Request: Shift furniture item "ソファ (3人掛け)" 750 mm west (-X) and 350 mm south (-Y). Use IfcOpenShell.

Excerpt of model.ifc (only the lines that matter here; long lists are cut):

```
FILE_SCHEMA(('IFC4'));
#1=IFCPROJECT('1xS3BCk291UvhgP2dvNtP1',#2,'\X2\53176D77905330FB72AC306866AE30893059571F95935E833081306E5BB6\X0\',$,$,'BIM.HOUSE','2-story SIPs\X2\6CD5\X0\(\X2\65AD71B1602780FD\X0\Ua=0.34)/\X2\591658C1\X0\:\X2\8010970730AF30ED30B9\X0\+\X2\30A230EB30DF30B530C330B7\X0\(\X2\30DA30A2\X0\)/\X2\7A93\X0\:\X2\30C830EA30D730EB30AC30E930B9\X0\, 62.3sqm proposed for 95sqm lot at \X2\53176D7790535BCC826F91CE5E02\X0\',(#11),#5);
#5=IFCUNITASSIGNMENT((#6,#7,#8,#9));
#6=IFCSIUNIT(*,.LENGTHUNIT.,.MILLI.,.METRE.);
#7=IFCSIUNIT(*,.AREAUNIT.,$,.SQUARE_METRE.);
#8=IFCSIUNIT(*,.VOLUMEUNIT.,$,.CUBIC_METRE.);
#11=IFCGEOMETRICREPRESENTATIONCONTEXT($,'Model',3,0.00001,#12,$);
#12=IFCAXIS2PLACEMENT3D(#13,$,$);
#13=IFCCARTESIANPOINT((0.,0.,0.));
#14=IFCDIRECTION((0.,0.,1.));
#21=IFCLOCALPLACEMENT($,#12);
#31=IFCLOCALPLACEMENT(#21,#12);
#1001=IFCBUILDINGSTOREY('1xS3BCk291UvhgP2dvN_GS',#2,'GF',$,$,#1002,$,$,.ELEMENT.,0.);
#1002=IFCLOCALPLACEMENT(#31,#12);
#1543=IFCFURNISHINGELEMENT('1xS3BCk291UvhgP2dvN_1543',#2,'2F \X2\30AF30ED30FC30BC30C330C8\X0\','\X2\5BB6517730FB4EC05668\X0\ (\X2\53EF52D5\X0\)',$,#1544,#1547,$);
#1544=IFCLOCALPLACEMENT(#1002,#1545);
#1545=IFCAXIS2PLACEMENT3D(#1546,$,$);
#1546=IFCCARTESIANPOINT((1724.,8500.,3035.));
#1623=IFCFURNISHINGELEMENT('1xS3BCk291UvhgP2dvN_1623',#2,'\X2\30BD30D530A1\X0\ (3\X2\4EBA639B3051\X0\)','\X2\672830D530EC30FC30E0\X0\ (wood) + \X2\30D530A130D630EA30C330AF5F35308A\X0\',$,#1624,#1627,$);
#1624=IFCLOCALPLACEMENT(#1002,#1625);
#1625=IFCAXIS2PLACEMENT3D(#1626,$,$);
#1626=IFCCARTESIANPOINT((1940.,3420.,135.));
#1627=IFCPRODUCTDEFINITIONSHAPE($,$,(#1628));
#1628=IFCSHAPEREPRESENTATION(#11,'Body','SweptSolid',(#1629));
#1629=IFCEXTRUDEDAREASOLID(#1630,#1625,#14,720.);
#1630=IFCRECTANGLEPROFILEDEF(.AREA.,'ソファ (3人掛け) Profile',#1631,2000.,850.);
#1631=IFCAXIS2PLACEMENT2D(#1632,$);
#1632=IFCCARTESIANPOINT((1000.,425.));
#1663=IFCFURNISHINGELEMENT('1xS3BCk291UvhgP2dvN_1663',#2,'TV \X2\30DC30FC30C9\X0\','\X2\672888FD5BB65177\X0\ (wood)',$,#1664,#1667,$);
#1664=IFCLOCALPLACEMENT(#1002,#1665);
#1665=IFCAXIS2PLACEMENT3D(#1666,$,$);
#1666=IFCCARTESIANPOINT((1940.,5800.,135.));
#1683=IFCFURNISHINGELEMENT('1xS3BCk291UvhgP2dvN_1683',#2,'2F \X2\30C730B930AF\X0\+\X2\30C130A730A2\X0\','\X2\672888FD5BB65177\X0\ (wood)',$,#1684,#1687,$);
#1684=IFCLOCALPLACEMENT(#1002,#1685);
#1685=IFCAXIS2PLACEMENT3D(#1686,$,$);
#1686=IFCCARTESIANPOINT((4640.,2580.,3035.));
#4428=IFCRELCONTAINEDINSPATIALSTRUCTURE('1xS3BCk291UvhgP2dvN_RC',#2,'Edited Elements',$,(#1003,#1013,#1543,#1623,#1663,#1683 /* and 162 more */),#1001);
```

```python
import ifcopenshell
import ifcopenshell.api.geometry
import ifcopenshell.util.placement

model = ifcopenshell.open("model.ifc")

item = model.by_id(1623)
matrix = ifcopenshell.util.placement.get_local_placement(item.ObjectPlacement)
matrix[0, 3] -= 750.0
matrix[1, 3] -= 350.0
ifcopenshell.api.geometry.edit_object_placement(model, product=item, matrix=matrix, is_si=False)

print(ifcopenshell.util.placement.get_local_placement(item.ObjectPlacement).round(3) + 0.0)

model.write("model-out.ifc")
```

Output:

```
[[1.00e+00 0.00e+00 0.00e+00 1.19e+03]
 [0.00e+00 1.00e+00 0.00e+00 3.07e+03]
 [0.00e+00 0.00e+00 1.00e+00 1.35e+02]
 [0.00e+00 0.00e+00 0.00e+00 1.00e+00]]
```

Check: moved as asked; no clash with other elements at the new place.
